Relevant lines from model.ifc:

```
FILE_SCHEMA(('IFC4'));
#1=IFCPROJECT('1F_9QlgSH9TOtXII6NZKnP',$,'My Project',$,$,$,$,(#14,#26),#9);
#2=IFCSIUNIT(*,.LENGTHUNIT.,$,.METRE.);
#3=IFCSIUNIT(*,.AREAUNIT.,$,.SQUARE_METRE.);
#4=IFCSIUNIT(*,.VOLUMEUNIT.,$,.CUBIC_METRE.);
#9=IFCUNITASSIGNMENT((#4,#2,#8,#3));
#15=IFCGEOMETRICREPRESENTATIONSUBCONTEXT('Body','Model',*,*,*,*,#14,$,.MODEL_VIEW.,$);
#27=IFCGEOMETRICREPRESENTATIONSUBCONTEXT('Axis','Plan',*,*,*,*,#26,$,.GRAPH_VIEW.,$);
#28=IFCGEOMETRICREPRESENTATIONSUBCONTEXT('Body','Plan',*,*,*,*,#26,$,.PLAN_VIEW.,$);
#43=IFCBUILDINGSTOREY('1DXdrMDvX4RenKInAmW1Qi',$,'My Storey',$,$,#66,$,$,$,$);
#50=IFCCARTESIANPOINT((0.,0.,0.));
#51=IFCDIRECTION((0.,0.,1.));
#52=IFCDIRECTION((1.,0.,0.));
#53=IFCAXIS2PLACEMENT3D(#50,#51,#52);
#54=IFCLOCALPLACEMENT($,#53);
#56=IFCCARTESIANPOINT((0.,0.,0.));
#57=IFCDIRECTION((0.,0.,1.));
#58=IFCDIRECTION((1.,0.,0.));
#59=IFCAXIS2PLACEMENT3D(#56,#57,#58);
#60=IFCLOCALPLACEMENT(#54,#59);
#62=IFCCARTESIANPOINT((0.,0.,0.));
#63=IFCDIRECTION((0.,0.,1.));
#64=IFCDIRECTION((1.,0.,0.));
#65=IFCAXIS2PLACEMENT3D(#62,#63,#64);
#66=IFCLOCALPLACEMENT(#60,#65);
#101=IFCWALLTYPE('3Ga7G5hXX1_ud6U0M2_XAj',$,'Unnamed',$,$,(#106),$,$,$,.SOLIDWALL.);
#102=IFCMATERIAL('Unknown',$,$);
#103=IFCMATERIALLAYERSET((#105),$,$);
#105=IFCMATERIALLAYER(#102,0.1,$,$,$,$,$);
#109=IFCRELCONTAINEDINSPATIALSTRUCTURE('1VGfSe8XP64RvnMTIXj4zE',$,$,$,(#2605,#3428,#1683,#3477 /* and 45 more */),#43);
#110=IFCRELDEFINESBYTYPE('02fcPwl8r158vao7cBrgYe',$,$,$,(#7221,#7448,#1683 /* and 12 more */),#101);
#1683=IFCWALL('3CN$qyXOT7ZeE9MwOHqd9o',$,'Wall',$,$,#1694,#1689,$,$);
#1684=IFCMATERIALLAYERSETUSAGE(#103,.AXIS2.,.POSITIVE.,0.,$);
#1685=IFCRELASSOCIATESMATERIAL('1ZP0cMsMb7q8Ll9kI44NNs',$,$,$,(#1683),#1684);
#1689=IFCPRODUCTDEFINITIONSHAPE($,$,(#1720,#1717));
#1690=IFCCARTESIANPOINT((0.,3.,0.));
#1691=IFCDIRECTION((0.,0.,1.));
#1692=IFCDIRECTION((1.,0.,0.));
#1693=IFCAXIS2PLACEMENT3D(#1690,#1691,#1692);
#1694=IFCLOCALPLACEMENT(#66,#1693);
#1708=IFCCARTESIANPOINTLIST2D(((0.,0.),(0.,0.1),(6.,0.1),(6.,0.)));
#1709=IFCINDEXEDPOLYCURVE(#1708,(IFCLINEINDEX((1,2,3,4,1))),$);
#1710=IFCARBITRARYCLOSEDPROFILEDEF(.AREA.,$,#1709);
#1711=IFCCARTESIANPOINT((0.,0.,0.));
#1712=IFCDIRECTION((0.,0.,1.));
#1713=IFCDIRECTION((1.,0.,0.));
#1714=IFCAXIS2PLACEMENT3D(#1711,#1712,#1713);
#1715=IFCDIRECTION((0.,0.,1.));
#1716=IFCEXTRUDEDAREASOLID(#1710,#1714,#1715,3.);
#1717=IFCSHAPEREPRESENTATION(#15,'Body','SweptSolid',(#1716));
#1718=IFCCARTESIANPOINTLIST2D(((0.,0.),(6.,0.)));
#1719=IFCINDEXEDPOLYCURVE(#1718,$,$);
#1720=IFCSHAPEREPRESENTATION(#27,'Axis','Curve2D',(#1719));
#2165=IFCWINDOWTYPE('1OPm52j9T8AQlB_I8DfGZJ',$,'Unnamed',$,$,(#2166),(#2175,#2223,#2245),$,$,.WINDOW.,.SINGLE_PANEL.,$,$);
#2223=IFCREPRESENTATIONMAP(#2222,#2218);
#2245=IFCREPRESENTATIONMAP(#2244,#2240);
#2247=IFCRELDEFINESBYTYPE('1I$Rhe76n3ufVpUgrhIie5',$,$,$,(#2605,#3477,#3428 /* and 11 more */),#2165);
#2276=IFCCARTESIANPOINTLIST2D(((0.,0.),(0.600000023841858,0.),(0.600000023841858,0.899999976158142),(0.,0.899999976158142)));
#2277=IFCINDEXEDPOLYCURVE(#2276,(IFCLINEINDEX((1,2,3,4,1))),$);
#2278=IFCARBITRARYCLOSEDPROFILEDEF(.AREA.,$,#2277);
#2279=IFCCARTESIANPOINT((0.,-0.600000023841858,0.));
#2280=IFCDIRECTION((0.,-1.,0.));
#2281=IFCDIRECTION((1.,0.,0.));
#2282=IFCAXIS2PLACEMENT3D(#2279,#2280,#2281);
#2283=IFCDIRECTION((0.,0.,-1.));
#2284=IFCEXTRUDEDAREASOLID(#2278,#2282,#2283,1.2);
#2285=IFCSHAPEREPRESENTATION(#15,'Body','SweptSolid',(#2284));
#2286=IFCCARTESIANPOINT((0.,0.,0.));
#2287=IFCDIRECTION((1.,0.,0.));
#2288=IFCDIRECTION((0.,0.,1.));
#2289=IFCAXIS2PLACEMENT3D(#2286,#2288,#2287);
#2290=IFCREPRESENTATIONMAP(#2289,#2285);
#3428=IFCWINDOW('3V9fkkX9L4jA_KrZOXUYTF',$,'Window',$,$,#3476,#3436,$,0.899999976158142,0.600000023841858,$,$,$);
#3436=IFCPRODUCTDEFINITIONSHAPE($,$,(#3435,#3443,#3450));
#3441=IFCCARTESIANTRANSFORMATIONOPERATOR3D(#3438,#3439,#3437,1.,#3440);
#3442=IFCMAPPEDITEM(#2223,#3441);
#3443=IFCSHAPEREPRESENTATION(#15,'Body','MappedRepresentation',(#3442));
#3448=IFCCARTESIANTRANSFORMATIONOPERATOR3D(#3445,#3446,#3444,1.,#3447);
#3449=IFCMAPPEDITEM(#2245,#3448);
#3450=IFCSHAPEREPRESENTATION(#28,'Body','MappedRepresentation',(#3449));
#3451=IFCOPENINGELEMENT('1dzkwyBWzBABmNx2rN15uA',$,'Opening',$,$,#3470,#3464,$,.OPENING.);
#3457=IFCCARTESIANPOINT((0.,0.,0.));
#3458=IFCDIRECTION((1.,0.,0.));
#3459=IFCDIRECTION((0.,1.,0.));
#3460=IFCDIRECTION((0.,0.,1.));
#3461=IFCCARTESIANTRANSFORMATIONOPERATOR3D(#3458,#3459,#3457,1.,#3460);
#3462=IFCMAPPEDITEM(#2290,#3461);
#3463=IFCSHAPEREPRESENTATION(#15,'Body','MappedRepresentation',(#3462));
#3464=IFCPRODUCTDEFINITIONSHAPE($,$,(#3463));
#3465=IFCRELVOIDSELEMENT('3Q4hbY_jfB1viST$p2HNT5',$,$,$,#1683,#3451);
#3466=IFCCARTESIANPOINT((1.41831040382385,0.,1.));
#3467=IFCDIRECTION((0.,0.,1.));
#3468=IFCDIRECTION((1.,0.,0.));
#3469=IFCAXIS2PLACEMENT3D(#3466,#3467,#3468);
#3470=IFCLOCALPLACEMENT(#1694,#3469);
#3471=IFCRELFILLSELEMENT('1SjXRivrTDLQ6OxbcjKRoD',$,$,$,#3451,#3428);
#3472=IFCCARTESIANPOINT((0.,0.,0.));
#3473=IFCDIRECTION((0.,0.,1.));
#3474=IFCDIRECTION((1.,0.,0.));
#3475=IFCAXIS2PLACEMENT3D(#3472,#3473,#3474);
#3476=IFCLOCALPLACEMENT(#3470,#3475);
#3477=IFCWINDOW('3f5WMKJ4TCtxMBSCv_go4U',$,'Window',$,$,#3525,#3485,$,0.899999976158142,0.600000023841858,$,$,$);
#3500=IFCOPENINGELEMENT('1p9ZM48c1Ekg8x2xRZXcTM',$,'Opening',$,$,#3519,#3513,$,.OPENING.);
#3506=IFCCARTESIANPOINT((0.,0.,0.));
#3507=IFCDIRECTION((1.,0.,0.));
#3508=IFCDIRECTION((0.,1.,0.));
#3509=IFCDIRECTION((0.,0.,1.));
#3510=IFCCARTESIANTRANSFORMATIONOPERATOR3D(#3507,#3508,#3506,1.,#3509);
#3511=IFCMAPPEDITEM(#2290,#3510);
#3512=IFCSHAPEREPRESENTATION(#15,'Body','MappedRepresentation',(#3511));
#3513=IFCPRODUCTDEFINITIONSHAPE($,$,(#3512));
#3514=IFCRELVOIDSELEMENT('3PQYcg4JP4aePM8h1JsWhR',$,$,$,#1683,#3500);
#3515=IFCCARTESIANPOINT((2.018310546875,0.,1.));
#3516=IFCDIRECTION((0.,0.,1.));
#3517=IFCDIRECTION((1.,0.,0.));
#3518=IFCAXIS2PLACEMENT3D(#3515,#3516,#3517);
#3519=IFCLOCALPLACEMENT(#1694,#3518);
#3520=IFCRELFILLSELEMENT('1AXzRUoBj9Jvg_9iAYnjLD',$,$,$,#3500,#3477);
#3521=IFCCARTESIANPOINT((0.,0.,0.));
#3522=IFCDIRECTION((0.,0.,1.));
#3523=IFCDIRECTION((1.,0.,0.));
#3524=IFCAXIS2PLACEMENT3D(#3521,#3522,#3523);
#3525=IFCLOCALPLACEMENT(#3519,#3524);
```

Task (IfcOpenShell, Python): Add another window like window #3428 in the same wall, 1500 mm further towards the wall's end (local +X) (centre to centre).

```python
import ifcopenshell
import ifcopenshell.api.feature
import ifcopenshell.api.geometry
import ifcopenshell.api.root
import ifcopenshell.geom
import ifcopenshell.util.element
import ifcopenshell.util.placement
import ifcopenshell.util.shape
import ifcopenshell.util.unit

model = ifcopenshell.open("model.ifc")
unit_scale = ifcopenshell.util.unit.calculate_unit_scale(model)
settings = ifcopenshell.geom.settings()


def volume(element):
    """Net volume in cubic metres, openings subtracted."""
    shape = ifcopenshell.geom.create_shape(settings, element)
    return ifcopenshell.util.shape.get_volume(shape.geometry)


window = model.by_guid("3V9fkkX9L4jA_KrZOXUYTF")
opening = window.FillsVoids[0].RelatingOpeningElement
wall = opening.VoidsElements[0].RelatingBuildingElement
before = volume(wall)
shift = ifcopenshell.util.placement.get_local_placement(wall.ObjectPlacement)[:3, 0] * 1.5 / unit_scale

# copy_class copies the void relationship, type, container and properties, but no geometry.
new_opening = ifcopenshell.api.root.copy_class(model, product=opening)
new_opening.Representation = ifcopenshell.util.element.copy_deep(
    model, opening.Representation, exclude=["IfcGeometricRepresentationContext", "IfcRepresentationMap"]
)
new_window = ifcopenshell.api.root.copy_class(model, product=window)
new_window.Representation = ifcopenshell.util.element.copy_deep(
    model, window.Representation, exclude=["IfcGeometricRepresentationContext", "IfcRepresentationMap"]
)
ifcopenshell.api.feature.add_filling(model, opening=new_opening, element=new_window)

for old, new in ((opening, new_opening), (window, new_window)):
    matrix = ifcopenshell.util.placement.get_local_placement(old.ObjectPlacement)
    matrix[:3, 3] += shift
    ifcopenshell.api.geometry.edit_object_placement(model, product=new, matrix=matrix, is_si=False)

after = volume(wall)

print(f"wall volume {before:.3f} -> {after:.3f} m3")

model.write("model_rev.ifc")
```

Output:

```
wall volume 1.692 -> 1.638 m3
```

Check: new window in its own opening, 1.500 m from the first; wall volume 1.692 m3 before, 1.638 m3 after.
